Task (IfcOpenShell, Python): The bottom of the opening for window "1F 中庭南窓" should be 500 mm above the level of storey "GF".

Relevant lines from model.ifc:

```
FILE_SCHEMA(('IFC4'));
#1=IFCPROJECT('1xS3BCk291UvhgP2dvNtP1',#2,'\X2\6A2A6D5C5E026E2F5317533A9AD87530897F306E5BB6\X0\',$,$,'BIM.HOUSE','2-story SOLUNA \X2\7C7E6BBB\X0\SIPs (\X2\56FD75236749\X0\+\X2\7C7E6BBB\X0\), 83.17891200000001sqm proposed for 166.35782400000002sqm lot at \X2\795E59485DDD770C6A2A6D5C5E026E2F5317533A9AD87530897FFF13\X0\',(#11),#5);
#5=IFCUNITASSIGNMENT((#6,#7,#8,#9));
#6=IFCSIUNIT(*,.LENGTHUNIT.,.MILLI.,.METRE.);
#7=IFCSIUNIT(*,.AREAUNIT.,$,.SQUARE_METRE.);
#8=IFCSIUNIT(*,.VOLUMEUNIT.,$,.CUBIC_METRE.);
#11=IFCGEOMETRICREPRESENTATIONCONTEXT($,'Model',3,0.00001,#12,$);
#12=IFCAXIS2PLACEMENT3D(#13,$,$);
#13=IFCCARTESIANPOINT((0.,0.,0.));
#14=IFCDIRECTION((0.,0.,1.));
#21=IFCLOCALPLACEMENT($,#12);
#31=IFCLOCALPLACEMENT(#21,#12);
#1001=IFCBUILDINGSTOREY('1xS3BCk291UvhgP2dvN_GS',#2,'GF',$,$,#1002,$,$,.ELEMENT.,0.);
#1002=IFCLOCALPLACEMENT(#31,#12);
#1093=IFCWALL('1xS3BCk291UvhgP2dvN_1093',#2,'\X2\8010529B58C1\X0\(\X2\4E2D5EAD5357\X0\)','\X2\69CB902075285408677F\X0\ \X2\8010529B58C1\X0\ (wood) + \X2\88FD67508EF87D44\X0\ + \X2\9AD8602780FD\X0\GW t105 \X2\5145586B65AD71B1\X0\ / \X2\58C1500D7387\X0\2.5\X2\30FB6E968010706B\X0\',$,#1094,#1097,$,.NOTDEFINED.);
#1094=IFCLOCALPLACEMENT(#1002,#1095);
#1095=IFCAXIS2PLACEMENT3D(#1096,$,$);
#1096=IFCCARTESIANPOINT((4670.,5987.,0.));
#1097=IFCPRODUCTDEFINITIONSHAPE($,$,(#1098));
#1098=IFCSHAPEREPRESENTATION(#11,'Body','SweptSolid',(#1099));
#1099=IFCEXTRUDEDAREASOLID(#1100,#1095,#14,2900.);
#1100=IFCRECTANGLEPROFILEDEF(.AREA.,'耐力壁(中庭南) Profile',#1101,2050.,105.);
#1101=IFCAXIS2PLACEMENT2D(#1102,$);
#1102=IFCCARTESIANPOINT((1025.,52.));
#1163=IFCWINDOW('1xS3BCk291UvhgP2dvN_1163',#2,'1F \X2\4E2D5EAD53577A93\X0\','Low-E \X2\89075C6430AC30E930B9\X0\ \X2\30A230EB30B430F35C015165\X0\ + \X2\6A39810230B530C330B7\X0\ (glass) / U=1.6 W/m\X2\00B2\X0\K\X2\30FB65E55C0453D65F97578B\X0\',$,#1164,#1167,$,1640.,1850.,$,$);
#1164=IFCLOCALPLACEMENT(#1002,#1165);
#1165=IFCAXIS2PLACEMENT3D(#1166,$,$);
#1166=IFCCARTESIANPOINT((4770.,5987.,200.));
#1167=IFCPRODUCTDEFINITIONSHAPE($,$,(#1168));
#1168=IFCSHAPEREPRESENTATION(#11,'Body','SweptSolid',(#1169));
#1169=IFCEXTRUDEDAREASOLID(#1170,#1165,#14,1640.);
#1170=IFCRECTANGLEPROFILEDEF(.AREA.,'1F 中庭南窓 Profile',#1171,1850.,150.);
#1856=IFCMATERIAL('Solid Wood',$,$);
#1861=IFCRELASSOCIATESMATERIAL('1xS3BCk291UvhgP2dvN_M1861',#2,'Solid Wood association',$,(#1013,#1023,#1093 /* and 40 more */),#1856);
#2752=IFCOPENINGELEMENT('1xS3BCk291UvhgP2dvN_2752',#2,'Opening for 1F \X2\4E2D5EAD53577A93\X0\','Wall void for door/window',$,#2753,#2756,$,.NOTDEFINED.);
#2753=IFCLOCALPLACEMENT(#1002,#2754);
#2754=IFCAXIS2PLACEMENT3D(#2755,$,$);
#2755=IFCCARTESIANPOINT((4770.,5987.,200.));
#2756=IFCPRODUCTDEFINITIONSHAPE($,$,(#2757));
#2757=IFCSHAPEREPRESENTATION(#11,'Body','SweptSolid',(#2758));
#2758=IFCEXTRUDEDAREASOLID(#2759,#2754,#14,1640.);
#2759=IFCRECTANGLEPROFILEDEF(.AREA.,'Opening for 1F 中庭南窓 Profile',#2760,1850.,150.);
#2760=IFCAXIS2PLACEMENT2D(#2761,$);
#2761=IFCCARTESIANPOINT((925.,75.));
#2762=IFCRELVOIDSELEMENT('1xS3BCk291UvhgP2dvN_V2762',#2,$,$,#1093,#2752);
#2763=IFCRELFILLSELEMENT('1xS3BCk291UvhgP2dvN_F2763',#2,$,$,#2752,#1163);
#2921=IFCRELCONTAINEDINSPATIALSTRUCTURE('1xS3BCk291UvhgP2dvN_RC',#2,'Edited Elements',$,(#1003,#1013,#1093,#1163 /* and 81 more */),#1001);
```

```python
import numpy as np
import ifcopenshell
import ifcopenshell.api.geometry
import ifcopenshell.geom
import ifcopenshell.util.element
import ifcopenshell.util.placement
import ifcopenshell.util.shape
import ifcopenshell.util.unit

model = ifcopenshell.open("model.ifc")
unit_scale = ifcopenshell.util.unit.calculate_unit_scale(model)

window = model.by_id(1163)
opening = window.FillsVoids[0].RelatingOpeningElement
storey = ifcopenshell.util.element.get_container(window, ifc_class="IfcBuildingStorey")
level = ifcopenshell.util.placement.get_local_placement(storey.ObjectPlacement)[2, 3]

# The opening's origin need not be at the sill, so measure its lowest point.
shape = ifcopenshell.geom.create_shape(ifcopenshell.geom.settings(), opening)
bottom = ifcopenshell.util.shape.get_shape_bottom_elevation(shape, shape.geometry) / unit_scale
dz = level + 500.0 - bottom

shift = np.array([0.0, 0.0, dz])
# The window is not placed relative to its opening, so move both.
for product in (opening, window):
    matrix = ifcopenshell.util.placement.get_local_placement(product.ObjectPlacement)
    matrix[:3, 3] += shift
    ifcopenshell.api.geometry.edit_object_placement(model, product=product, matrix=matrix, is_si=False)

print(f"moved by {dz * unit_scale:+.3f} m")

model.write("model_rev.ifc")
```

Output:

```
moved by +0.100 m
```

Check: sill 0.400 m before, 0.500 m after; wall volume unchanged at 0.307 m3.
